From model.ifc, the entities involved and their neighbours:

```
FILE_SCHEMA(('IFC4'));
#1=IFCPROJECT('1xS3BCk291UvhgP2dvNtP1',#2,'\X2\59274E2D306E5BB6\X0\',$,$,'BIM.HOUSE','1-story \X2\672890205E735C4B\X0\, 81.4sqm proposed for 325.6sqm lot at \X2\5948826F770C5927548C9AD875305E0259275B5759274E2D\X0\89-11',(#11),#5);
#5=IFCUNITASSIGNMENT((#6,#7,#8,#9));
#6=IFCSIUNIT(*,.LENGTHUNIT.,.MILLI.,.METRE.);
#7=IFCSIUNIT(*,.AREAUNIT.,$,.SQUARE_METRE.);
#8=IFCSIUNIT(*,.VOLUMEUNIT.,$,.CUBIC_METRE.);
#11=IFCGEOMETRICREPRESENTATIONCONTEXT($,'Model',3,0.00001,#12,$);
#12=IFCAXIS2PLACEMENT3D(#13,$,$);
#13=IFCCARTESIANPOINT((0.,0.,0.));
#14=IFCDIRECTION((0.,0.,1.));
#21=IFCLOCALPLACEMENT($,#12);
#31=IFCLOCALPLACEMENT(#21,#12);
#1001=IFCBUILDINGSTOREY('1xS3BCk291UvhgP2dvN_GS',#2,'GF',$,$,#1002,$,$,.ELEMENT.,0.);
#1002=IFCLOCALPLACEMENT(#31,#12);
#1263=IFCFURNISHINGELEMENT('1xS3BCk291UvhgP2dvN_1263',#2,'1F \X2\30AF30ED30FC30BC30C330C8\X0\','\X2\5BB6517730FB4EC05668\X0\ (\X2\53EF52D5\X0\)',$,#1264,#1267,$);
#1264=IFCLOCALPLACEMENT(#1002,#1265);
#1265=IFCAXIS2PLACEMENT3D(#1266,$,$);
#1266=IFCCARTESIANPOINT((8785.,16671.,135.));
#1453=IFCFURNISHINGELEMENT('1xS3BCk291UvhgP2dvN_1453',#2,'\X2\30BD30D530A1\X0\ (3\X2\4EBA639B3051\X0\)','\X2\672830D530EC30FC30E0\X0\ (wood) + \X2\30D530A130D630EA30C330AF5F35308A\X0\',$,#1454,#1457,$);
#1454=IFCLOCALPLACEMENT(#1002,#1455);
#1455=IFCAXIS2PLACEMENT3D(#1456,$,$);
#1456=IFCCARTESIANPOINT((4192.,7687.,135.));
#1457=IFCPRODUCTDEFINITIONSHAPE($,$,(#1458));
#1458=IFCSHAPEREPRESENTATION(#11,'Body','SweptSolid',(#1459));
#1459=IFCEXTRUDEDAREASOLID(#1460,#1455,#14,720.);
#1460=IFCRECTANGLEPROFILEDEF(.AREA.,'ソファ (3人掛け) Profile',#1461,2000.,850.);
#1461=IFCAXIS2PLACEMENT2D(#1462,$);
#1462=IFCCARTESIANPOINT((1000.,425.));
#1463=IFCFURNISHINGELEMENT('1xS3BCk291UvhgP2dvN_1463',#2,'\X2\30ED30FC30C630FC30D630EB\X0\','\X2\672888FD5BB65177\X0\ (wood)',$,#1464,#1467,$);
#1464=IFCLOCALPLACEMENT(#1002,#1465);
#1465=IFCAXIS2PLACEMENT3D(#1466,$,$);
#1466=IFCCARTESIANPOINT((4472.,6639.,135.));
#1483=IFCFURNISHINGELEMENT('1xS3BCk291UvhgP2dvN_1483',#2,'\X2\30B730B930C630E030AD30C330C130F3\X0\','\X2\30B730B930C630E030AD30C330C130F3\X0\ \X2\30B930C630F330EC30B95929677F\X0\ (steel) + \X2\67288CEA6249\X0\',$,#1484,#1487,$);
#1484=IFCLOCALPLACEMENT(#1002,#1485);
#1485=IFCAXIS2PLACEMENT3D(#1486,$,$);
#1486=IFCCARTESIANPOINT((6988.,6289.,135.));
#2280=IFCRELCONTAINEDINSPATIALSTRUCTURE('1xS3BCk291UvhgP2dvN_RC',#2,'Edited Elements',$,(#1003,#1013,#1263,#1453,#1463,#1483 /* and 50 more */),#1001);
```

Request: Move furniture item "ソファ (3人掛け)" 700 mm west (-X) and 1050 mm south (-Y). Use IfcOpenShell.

```python
import ifcopenshell
import ifcopenshell.api.geometry
import ifcopenshell.util.placement
import ifcopenshell.util.unit

model = ifcopenshell.open("model.ifc")
unit_scale = ifcopenshell.util.unit.calculate_unit_scale(model)

item = model.by_guid("1xS3BCk291UvhgP2dvN_1453")
matrix = ifcopenshell.util.placement.get_local_placement(item.ObjectPlacement)
matrix[0, 3] -= 0.7 / unit_scale
matrix[1, 3] -= 1.05 / unit_scale
ifcopenshell.api.geometry.edit_object_placement(model, product=item, matrix=matrix, is_si=False)

print(ifcopenshell.util.placement.get_local_placement(item.ObjectPlacement).round(3) + 0.0)

model.write("model_v2.ifc")
```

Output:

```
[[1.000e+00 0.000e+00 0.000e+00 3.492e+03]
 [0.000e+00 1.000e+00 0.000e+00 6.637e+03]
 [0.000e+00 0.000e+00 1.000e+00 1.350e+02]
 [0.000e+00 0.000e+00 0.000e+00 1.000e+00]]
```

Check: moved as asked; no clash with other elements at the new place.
